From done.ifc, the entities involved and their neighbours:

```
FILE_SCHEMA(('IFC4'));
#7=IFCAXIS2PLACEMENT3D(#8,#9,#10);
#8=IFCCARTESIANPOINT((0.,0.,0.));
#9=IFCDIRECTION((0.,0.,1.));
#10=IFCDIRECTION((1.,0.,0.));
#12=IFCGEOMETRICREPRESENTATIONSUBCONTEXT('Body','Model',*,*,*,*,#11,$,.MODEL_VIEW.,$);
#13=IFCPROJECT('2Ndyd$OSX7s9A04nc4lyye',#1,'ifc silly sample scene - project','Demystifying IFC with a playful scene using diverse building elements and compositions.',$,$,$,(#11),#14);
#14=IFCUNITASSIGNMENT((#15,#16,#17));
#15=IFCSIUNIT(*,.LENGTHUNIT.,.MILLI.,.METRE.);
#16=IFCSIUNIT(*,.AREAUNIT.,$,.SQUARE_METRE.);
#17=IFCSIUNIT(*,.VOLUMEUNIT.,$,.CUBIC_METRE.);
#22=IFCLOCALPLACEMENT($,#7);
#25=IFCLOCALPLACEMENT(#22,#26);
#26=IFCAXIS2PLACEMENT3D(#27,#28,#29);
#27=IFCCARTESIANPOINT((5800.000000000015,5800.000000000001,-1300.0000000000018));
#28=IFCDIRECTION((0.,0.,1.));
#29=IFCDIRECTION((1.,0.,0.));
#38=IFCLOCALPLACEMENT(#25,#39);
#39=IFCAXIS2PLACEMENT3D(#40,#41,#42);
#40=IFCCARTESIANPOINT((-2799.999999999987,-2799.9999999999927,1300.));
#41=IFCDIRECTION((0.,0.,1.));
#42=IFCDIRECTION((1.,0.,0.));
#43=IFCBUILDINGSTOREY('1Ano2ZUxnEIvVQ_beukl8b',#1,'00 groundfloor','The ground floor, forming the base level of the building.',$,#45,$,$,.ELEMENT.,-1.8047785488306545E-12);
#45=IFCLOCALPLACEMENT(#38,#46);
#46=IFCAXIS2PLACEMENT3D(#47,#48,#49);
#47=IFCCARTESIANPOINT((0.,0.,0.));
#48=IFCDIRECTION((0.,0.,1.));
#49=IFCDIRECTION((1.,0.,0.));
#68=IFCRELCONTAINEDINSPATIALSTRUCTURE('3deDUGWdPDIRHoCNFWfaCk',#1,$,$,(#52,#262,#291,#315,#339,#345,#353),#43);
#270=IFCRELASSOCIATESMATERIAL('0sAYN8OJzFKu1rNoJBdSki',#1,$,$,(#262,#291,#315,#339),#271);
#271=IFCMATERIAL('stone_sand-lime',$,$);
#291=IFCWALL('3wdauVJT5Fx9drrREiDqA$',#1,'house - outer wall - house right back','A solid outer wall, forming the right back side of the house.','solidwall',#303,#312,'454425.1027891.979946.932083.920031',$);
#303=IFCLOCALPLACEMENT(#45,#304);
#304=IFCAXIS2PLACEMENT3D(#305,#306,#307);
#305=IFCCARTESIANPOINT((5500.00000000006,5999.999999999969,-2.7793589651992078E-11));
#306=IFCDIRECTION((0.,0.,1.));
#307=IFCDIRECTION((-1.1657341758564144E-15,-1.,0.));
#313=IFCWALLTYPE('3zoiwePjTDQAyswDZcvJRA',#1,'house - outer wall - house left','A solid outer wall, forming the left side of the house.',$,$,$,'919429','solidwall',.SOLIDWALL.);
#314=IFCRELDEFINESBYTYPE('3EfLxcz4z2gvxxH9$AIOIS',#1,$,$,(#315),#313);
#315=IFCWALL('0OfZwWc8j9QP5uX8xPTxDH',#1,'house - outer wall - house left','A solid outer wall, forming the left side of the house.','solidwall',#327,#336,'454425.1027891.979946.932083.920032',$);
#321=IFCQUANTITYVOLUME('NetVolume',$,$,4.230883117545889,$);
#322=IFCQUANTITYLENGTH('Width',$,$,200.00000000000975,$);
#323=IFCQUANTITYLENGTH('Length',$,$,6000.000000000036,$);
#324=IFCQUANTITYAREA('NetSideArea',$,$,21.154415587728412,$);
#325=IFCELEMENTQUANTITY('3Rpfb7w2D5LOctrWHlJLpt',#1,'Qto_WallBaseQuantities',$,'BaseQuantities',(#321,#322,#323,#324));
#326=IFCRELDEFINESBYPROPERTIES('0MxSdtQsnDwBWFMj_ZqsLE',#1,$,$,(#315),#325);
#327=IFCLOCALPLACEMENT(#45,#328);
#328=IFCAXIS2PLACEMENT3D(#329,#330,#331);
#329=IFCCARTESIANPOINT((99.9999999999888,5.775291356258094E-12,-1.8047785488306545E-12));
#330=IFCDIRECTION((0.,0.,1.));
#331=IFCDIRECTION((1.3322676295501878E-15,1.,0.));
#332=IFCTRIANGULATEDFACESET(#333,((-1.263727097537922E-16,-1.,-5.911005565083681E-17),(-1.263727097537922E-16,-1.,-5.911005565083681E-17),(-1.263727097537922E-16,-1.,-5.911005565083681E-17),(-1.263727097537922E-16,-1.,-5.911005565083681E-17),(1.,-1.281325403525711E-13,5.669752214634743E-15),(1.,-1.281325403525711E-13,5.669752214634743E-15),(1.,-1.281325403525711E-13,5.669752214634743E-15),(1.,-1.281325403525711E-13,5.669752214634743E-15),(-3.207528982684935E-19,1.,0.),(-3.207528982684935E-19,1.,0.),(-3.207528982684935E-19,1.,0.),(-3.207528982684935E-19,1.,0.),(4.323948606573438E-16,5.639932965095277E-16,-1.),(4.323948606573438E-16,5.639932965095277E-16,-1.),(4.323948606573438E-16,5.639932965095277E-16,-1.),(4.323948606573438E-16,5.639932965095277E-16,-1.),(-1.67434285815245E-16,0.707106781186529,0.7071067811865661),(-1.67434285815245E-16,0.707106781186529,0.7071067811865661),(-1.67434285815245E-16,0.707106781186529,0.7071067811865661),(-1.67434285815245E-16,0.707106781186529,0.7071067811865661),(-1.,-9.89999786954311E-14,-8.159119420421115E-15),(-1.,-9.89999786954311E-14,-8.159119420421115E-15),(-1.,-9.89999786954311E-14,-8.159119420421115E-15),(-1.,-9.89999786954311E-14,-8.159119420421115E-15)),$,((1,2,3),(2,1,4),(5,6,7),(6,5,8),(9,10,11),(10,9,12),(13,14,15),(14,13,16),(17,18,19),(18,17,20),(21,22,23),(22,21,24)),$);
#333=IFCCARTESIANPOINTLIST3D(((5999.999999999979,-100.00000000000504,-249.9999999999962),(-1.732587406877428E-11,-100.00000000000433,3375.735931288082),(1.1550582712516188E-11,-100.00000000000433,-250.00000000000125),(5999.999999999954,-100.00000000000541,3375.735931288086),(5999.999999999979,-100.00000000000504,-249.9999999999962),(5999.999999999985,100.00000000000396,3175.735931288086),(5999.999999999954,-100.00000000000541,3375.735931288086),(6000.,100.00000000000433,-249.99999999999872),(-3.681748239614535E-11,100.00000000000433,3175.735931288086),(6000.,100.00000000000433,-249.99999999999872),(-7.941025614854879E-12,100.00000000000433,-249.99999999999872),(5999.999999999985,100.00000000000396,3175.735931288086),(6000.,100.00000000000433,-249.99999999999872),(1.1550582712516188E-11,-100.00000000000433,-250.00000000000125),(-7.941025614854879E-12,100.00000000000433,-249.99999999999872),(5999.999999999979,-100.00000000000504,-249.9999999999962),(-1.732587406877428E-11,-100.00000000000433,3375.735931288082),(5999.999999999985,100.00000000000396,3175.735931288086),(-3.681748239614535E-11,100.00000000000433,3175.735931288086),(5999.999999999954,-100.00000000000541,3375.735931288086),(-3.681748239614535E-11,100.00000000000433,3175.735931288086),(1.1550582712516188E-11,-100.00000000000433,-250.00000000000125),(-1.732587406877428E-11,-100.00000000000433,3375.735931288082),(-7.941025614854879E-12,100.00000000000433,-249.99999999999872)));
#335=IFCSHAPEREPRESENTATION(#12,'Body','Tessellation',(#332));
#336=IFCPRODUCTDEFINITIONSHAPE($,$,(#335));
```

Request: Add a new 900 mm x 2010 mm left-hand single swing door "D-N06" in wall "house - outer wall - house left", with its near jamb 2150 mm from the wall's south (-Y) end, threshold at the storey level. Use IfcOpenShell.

```python
import numpy as np
import ifcopenshell
import ifcopenshell.api.feature
import ifcopenshell.api.geometry
import ifcopenshell.api.pset
import ifcopenshell.api.root
import ifcopenshell.api.spatial
import ifcopenshell.geom
import ifcopenshell.util.element
import ifcopenshell.util.placement
import ifcopenshell.util.representation
import ifcopenshell.util.shape
import ifcopenshell.util.unit

model = ifcopenshell.open("done.ifc")
unit_scale = ifcopenshell.util.unit.calculate_unit_scale(model)
area_scale = ifcopenshell.util.unit.calculate_unit_scale(model, "AREAUNIT")
volume_scale = ifcopenshell.util.unit.calculate_unit_scale(model, "VOLUMEUNIT")
settings = ifcopenshell.geom.settings()


def volume(element):
    """Net volume in cubic metres, openings subtracted."""
    shape = ifcopenshell.geom.create_shape(settings, element)
    return ifcopenshell.util.shape.get_volume(shape.geometry)


wall = model.by_guid("0OfZwWc8j9QP5uX8xPTxDH")
storey = ifcopenshell.util.element.get_container(wall, ifc_class="IfcBuildingStorey")
context = ifcopenshell.util.representation.get_context(model, "Model", "Body", "MODEL_VIEW")
before = volume(wall)

width, height, from_end, sill = 0.9, 2.01, 2.15, 0.0  # metres

# The wall runs along its own X axis, and the end named is its -X end.
wall_shape = ifcopenshell.geom.create_shape(settings, wall)
x, y, z = ifcopenshell.util.shape.get_vertices(wall_shape.geometry).T
start = x.min() + from_end
face, thickness = float(y.min()), float(y.max() - y.min())
wall_matrix = ifcopenshell.util.placement.get_local_placement(wall.ObjectPlacement)
level = ifcopenshell.util.placement.get_local_placement(storey.ObjectPlacement)[2, 3]


def in_wall(x, y):
    """Placement at x, y metres in the wall's axes, at sill height."""
    matrix = wall_matrix.copy()
    matrix[:, 3] = wall_matrix @ np.array([x / unit_scale, y / unit_scale, 0.0, 1.0])
    matrix[2, 3] = level + sill / unit_scale
    return matrix


# Opening: a box that overshoots both wall faces by 50 mm.
opening = ifcopenshell.api.root.create_entity(model, ifc_class="IfcOpeningElement", predefined_type="OPENING")
box = ifcopenshell.api.geometry.add_wall_representation(
    model, context=context, length=width, height=height, thickness=thickness + 0.1
)
ifcopenshell.api.geometry.assign_representation(model, product=opening, representation=box)
ifcopenshell.api.geometry.edit_object_placement(model, product=opening, matrix=in_wall(start, face - 0.05), is_si=False)
ifcopenshell.api.feature.add_feature(model, feature=opening, element=wall)

door = ifcopenshell.api.root.create_entity(model, ifc_class="IfcDoor", name="D-N06", predefined_type="DOOR")
door.OverallWidth, door.OverallHeight = width / unit_scale, height / unit_scale
door.OperationType = "SINGLE_SWING_LEFT"
body = ifcopenshell.api.geometry.add_door_representation(
    model,
    context=context,
    overall_width=door.OverallWidth,
    overall_height=door.OverallHeight,
    operation_type="SINGLE_SWING_LEFT",
    lining_properties={"LiningDepth": thickness / unit_scale, "ThresholdDepth": thickness / unit_scale},
)
ifcopenshell.api.geometry.assign_representation(model, product=door, representation=body)
ifcopenshell.api.spatial.assign_container(model, products=[door], relating_structure=storey)
ifcopenshell.api.feature.add_filling(model, opening=opening, element=door)

# The lining spans the wall, so the door starts at the wall face.
ifcopenshell.api.geometry.edit_object_placement(model, product=door, matrix=in_wall(start, face), is_si=False)

after = volume(wall)

# Update the wall's stored quantities.
qto = model.by_id(ifcopenshell.util.element.get_pset(wall, "Qto_WallBaseQuantities", should_inherit=False)["id"])
ifcopenshell.api.pset.edit_qto(model, qto=qto, properties={
    "NetVolume": after / volume_scale,
    "NetSideArea": after / thickness / area_scale,
})

print(f"wall volume {before:.3f} -> {after:.3f} m3")

model.write("done_rev.ifc")
```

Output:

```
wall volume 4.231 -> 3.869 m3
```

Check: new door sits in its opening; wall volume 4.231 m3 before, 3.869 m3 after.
